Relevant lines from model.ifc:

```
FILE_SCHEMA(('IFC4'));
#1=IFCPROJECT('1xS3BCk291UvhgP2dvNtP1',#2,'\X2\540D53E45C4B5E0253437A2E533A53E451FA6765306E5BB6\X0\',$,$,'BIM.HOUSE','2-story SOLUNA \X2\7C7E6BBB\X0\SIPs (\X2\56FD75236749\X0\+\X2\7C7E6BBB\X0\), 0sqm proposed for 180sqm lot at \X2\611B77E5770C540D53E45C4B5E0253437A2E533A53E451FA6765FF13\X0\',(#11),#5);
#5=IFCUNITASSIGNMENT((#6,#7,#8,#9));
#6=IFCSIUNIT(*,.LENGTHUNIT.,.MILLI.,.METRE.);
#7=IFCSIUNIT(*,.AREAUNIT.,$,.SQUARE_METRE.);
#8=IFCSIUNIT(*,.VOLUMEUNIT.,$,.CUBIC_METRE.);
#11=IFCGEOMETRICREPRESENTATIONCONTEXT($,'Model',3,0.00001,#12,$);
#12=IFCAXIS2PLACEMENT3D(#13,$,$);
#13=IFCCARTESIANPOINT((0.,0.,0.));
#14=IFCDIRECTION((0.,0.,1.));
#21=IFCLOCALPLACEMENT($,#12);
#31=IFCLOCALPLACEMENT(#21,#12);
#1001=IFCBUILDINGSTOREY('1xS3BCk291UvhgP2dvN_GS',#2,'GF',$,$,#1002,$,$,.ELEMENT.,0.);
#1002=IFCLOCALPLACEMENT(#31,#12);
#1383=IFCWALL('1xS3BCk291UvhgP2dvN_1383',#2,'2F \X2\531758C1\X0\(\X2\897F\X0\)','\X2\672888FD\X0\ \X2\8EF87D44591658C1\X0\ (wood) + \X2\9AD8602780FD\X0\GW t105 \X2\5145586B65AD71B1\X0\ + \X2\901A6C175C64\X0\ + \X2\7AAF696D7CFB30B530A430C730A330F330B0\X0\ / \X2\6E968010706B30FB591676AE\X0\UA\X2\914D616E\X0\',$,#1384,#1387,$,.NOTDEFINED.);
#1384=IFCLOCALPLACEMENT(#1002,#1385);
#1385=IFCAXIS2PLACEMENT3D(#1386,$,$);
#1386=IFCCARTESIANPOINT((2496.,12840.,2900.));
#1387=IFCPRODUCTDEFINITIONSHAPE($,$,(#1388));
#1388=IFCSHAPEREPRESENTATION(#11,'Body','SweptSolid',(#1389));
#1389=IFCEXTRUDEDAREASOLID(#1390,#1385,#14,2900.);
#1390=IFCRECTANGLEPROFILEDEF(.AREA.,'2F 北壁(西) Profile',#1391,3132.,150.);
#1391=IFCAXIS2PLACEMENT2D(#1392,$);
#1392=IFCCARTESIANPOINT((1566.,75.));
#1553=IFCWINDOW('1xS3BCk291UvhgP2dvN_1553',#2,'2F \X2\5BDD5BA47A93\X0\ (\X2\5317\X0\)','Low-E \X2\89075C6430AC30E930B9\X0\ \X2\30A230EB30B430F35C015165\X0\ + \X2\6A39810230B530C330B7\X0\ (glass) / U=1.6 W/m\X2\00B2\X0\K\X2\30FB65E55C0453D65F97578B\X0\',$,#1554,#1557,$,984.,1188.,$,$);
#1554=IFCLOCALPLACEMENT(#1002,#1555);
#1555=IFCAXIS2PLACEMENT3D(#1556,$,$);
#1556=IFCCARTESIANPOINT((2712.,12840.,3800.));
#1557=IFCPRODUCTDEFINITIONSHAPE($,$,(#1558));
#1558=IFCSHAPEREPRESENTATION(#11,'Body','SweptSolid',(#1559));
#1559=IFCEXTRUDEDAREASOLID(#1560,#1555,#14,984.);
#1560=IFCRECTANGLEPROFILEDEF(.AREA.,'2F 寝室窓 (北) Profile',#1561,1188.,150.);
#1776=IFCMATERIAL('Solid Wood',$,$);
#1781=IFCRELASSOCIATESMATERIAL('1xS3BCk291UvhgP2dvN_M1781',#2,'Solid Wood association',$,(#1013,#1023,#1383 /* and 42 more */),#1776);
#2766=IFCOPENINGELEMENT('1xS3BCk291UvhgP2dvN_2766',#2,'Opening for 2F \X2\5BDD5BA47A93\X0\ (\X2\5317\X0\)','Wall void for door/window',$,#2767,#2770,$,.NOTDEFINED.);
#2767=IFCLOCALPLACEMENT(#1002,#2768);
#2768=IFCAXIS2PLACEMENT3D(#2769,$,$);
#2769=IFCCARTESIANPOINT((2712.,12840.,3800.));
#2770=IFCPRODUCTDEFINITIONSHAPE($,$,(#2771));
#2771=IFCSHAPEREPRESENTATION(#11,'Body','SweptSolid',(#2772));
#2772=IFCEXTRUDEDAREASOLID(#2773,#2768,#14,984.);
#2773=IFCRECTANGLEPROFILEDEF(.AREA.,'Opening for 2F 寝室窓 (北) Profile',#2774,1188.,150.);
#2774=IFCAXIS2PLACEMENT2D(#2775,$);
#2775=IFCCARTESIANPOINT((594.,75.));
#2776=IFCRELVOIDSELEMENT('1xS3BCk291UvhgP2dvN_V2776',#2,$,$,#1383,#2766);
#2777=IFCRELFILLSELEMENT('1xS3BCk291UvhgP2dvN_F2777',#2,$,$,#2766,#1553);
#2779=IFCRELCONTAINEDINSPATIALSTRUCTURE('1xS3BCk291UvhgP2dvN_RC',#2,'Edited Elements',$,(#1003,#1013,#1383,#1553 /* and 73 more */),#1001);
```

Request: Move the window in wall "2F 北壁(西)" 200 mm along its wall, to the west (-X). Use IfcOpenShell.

```python
import ifcopenshell
import ifcopenshell.api.geometry
import ifcopenshell.util.placement
import ifcopenshell.util.unit

model = ifcopenshell.open("model.ifc")
unit_scale = ifcopenshell.util.unit.calculate_unit_scale(model)

window = model.by_id(1553)
opening = window.FillsVoids[0].RelatingOpeningElement
wall = opening.VoidsElements[0].RelatingBuildingElement

wall_matrix = ifcopenshell.util.placement.get_local_placement(wall.ObjectPlacement)
shift = wall_matrix[:3, 0] * -0.2 / unit_scale
before = ifcopenshell.util.placement.get_local_placement(window.ObjectPlacement)[:3, 3].copy()

# The window is not placed relative to its opening, so move both.
for product in (opening, window):
    matrix = ifcopenshell.util.placement.get_local_placement(product.ObjectPlacement)
    matrix[:3, 3] += shift
    ifcopenshell.api.geometry.edit_object_placement(model, product=product, matrix=matrix, is_si=False)

after = ifcopenshell.util.placement.get_local_placement(window.ObjectPlacement)[:3, 3]
print("window moved by", (after - before).round(3) + 0.0)

model.write("model-out.ifc")
```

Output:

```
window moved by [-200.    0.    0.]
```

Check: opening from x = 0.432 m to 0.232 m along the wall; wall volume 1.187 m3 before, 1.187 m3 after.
